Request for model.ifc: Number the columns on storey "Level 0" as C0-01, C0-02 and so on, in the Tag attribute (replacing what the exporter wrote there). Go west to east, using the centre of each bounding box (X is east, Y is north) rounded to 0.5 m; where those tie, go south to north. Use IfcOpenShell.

First a look at what the model holds.

```python
import ifcopenshell
import ifcopenshell.util.element
import ifcopenshell.util.placement

model = ifcopenshell.open("model.ifc")
print(model.schema)
storey = next(s for s in model.by_type("IfcBuildingStorey") if s.Name == "Level 0")
columns = [e for e in ifcopenshell.util.element.get_decomposition(storey) if e.is_a("IfcColumn")]
for e in sorted(columns, key=lambda e: e.id()):
    origin = ifcopenshell.util.placement.get_local_placement(e.ObjectPlacement)[:3, 3]
    print(e.id(), e.Tag, e.Name, origin.round(2) + 0.0, sep=" | ")
```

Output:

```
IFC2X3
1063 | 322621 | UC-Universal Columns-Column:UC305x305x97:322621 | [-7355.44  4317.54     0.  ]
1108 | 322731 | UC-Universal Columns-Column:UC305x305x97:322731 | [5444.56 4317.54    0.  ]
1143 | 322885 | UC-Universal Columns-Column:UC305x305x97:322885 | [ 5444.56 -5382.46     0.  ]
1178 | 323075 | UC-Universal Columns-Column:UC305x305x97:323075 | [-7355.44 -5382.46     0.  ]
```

```python
import ifcopenshell
import ifcopenshell.geom
import ifcopenshell.util.element
import ifcopenshell.util.shape

model = ifcopenshell.open("model.ifc")
settings = ifcopenshell.geom.settings()
settings.set("use-world-coords", True)


def centre(element):
    shape = ifcopenshell.geom.create_shape(settings, element)
    return ifcopenshell.util.shape.get_bbox_centroid(shape.geometry)


storey = next(s for s in model.by_type("IfcBuildingStorey") if s.Name == "Level 0")
columns = [e for e in ifcopenshell.util.element.get_decomposition(storey) if e.is_a("IfcColumn")]

# Insertion points can sit at a corner or the storey origin, so sort by the geometry (in metres).
centres = {e: centre(e) for e in columns}
columns.sort(key=lambda e: (round(centres[e][0] / 0.5), centres[e][1]))

for i, e in enumerate(columns, start=1):
    number = f"C0-{i:02d}"
    e.Tag = number
    print(e.id(), number)

model.write("model_updated.ifc")
```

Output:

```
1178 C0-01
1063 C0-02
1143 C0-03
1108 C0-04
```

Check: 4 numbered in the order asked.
